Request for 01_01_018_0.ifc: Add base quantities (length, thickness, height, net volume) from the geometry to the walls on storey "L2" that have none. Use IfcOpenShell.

First a look at what the model holds.

```python
import ifcopenshell
import ifcopenshell.util.element
import ifcopenshell.util.unit

model = ifcopenshell.open("01_01_018_0.ifc")
print(model.schema)
for unit_type in ("LENGTHUNIT", "AREAUNIT", "VOLUMEUNIT"):
    print(unit_type, ifcopenshell.util.unit.calculate_unit_scale(model, unit_type))
storey = next(s for s in model.by_type("IfcBuildingStorey") if s.Name == "L2")
walls = [e for e in ifcopenshell.util.element.get_decomposition(storey) if e.is_a("IfcWall")]
for e in sorted(walls, key=lambda e: e.id()):
    print(e.id(), e.is_a(), e.Name, list(ifcopenshell.util.element.get_psets(e, qtos_only=True)), sep=" | ")
```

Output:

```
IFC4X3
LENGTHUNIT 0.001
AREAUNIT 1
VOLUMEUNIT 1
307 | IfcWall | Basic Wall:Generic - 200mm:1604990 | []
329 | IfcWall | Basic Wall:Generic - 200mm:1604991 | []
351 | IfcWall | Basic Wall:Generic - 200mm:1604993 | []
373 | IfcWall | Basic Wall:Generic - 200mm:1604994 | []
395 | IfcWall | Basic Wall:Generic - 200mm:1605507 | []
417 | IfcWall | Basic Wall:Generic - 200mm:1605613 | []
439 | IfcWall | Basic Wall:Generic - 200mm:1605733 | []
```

```python
import ifcopenshell
import ifcopenshell.api.pset
import ifcopenshell.geom
import ifcopenshell.util.element
import ifcopenshell.util.shape
import ifcopenshell.util.unit

model = ifcopenshell.open("01_01_018_0.ifc")
unit_scale = ifcopenshell.util.unit.calculate_unit_scale(model)
volume_scale = ifcopenshell.util.unit.calculate_unit_scale(model, "VOLUMEUNIT")
settings = ifcopenshell.geom.settings()

storey = next(s for s in model.by_type("IfcBuildingStorey") if s.Name == "L2")
walls = [e for e in ifcopenshell.util.element.get_decomposition(storey) if e.is_a("IfcWall")]

for e in sorted(walls, key=lambda e: e.id()):
    if ifcopenshell.util.element.get_psets(e, qtos_only=True, should_inherit=False):
        continue
    # Geometry comes back in metres, in the element's own axes.
    shape = ifcopenshell.geom.create_shape(settings, e)
    values = {
        "Length": ifcopenshell.util.shape.get_x(shape.geometry) / unit_scale,
        "Width": ifcopenshell.util.shape.get_y(shape.geometry) / unit_scale,
        "Height": ifcopenshell.util.shape.get_z(shape.geometry) / unit_scale,
        "NetVolume": ifcopenshell.util.shape.get_volume(shape.geometry) / volume_scale,
    }
    qto = ifcopenshell.api.pset.add_qto(model, product=e, name="Qto_WallBaseQuantities")
    ifcopenshell.api.pset.edit_qto(model, qto=qto, properties=values)
    print(e.id(), {k: round(v, 3) for k, v in values.items()})

model.write("01_01_018_0_v2.ifc")
```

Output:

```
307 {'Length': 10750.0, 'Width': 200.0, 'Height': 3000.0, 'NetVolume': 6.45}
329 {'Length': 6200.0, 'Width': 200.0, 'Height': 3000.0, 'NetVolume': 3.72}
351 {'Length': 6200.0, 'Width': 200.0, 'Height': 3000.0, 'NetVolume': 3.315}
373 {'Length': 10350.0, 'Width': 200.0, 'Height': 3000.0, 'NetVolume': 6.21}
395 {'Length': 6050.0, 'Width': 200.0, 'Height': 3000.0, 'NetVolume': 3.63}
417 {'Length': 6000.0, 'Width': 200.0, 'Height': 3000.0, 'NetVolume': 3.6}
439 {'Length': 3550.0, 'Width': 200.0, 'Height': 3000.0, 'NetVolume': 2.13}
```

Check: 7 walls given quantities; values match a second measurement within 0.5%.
